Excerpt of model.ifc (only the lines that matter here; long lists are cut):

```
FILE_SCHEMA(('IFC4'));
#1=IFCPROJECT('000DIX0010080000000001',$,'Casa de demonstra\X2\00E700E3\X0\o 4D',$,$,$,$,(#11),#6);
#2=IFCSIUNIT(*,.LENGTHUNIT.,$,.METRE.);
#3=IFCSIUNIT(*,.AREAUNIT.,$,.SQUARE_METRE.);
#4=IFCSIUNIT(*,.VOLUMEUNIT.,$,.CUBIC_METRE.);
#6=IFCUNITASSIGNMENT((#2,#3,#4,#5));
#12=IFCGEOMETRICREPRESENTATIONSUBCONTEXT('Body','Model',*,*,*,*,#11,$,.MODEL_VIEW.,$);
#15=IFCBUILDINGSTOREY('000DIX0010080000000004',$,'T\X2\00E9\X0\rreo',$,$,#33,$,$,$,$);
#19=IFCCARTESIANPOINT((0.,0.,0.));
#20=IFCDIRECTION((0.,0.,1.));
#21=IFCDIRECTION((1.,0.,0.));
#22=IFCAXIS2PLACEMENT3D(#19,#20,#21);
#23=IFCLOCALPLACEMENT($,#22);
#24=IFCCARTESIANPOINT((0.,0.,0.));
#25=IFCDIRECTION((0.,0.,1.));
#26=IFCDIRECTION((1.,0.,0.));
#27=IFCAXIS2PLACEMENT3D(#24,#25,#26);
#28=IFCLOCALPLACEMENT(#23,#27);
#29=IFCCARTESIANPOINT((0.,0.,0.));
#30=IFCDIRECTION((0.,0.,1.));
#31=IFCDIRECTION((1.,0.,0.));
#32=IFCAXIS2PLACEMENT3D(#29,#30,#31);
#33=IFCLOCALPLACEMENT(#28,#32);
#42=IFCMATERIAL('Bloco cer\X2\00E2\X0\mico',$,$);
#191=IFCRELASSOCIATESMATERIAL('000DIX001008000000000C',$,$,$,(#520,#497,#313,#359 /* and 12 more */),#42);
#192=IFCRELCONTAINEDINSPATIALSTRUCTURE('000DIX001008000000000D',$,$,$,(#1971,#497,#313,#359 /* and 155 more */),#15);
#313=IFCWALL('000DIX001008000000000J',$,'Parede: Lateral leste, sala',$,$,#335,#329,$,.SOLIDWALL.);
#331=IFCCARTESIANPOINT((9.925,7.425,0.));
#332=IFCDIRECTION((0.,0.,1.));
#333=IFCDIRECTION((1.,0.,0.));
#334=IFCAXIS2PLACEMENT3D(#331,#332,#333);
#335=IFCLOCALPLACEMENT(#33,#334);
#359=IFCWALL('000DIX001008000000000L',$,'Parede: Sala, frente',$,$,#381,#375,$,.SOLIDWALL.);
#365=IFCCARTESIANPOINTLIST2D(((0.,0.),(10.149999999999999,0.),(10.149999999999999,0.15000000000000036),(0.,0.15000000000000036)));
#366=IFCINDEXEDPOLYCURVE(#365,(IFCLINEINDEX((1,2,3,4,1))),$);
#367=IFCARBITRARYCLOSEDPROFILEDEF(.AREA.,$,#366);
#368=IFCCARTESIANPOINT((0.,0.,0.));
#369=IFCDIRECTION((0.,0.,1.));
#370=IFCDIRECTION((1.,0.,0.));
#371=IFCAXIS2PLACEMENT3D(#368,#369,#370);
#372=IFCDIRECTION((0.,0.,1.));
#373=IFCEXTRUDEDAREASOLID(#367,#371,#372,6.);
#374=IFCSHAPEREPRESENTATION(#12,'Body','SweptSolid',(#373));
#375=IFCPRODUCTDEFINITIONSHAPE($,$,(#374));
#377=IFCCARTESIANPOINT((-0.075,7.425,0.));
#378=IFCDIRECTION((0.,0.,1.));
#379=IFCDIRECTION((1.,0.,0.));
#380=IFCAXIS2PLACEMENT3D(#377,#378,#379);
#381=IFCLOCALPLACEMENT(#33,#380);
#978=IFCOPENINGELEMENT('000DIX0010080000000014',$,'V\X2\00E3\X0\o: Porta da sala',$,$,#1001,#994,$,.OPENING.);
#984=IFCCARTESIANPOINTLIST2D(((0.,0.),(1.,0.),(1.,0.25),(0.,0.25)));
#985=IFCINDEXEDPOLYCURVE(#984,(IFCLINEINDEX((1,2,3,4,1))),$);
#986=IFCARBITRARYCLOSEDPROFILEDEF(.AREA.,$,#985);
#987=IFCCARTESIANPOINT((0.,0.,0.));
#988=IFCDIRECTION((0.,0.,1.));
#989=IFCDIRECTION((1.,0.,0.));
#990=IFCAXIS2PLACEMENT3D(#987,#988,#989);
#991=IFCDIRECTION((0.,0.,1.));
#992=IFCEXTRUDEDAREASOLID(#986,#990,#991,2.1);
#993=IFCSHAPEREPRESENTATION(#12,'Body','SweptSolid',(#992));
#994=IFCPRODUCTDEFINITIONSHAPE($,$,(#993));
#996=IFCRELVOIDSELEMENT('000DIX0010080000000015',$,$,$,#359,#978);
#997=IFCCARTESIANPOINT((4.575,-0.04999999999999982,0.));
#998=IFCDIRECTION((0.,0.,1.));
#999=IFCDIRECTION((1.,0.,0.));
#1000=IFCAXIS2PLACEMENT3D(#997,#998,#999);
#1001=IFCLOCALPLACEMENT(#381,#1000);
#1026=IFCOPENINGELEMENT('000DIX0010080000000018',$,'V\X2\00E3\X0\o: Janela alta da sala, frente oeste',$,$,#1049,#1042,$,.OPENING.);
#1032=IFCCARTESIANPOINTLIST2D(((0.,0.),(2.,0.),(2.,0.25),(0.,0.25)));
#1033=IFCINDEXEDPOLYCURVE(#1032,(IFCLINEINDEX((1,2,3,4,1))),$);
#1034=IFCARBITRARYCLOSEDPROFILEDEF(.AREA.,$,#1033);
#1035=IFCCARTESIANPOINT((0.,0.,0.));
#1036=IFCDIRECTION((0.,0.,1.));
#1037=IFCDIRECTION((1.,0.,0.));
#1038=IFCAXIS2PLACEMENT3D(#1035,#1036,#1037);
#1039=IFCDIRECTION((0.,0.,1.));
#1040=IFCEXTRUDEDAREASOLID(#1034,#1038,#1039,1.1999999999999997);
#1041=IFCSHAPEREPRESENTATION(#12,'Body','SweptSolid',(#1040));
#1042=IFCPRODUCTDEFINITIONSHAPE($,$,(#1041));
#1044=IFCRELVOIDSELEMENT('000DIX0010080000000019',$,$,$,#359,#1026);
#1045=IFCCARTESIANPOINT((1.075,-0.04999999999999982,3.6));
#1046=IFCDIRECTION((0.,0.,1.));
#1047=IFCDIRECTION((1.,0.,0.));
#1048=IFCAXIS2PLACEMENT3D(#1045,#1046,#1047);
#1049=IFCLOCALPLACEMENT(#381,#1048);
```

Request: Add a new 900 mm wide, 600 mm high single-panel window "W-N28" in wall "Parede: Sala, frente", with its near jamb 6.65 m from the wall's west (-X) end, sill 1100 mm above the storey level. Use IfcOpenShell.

```python
import numpy as np
import ifcopenshell
import ifcopenshell.api.feature
import ifcopenshell.api.geometry
import ifcopenshell.api.root
import ifcopenshell.api.spatial
import ifcopenshell.geom
import ifcopenshell.util.element
import ifcopenshell.util.placement
import ifcopenshell.util.representation
import ifcopenshell.util.shape
import ifcopenshell.util.unit

model = ifcopenshell.open("model.ifc")
unit_scale = ifcopenshell.util.unit.calculate_unit_scale(model)
settings = ifcopenshell.geom.settings()


def volume(element):
    """Net volume in cubic metres, openings subtracted."""
    shape = ifcopenshell.geom.create_shape(settings, element)
    return ifcopenshell.util.shape.get_volume(shape.geometry)


wall = model.by_guid("000DIX001008000000000L")
storey = ifcopenshell.util.element.get_container(wall, ifc_class="IfcBuildingStorey")
context = ifcopenshell.util.representation.get_context(model, "Model", "Body", "MODEL_VIEW")
before = volume(wall)

width, height, from_end, sill = 0.9, 0.6, 6.65, 1.1  # metres

# The wall runs along its own X axis, and the end named is its -X end.
wall_shape = ifcopenshell.geom.create_shape(settings, wall)
x, y, z = ifcopenshell.util.shape.get_vertices(wall_shape.geometry).T
start = x.min() + from_end
face, thickness = float(y.min()), float(y.max() - y.min())
wall_matrix = ifcopenshell.util.placement.get_local_placement(wall.ObjectPlacement)
level = ifcopenshell.util.placement.get_local_placement(storey.ObjectPlacement)[2, 3]


def in_wall(x, y):
    """Placement at x, y metres in the wall's axes, at sill height."""
    matrix = wall_matrix.copy()
    matrix[:, 3] = wall_matrix @ np.array([x / unit_scale, y / unit_scale, 0.0, 1.0])
    matrix[2, 3] = level + sill / unit_scale
    return matrix


# Opening: a box that overshoots both wall faces by 50 mm.
opening = ifcopenshell.api.root.create_entity(model, ifc_class="IfcOpeningElement", predefined_type="OPENING")
box = ifcopenshell.api.geometry.add_wall_representation(
    model, context=context, length=width, height=height, thickness=thickness + 0.1
)
ifcopenshell.api.geometry.assign_representation(model, product=opening, representation=box)
ifcopenshell.api.geometry.edit_object_placement(model, product=opening, matrix=in_wall(start, face - 0.05), is_si=False)
ifcopenshell.api.feature.add_feature(model, feature=opening, element=wall)

window = ifcopenshell.api.root.create_entity(model, ifc_class="IfcWindow", name="W-N28", predefined_type="WINDOW")
window.OverallWidth, window.OverallHeight = width / unit_scale, height / unit_scale
window.PartitioningType = "SINGLE_PANEL"
body = ifcopenshell.api.geometry.add_window_representation(
    model,
    context=context,
    overall_width=window.OverallWidth,
    overall_height=window.OverallHeight,
    partition_type="SINGLE_PANEL",
)
ifcopenshell.api.geometry.assign_representation(model, product=window, representation=body)
ifcopenshell.api.spatial.assign_container(model, products=[window], relating_structure=storey)
ifcopenshell.api.feature.add_filling(model, opening=opening, element=window)

# Centre the window in the wall's thickness.
ifcopenshell.api.geometry.edit_object_placement(model, product=window, matrix=in_wall(start, face), is_si=False)
window_shape = ifcopenshell.geom.create_shape(settings, window)
depth = ifcopenshell.util.shape.get_vertices(window_shape.geometry)[:, 1]
offset = face + thickness / 2 - (depth.min() + depth.max()) / 2
ifcopenshell.api.geometry.edit_object_placement(model, product=window, matrix=in_wall(start, offset), is_si=False)

after = volume(wall)

print(f"wall volume {before:.3f} -> {after:.3f} m3")

model.write("model_updated.ifc")
```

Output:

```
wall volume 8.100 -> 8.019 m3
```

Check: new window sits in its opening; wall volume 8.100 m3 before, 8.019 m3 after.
